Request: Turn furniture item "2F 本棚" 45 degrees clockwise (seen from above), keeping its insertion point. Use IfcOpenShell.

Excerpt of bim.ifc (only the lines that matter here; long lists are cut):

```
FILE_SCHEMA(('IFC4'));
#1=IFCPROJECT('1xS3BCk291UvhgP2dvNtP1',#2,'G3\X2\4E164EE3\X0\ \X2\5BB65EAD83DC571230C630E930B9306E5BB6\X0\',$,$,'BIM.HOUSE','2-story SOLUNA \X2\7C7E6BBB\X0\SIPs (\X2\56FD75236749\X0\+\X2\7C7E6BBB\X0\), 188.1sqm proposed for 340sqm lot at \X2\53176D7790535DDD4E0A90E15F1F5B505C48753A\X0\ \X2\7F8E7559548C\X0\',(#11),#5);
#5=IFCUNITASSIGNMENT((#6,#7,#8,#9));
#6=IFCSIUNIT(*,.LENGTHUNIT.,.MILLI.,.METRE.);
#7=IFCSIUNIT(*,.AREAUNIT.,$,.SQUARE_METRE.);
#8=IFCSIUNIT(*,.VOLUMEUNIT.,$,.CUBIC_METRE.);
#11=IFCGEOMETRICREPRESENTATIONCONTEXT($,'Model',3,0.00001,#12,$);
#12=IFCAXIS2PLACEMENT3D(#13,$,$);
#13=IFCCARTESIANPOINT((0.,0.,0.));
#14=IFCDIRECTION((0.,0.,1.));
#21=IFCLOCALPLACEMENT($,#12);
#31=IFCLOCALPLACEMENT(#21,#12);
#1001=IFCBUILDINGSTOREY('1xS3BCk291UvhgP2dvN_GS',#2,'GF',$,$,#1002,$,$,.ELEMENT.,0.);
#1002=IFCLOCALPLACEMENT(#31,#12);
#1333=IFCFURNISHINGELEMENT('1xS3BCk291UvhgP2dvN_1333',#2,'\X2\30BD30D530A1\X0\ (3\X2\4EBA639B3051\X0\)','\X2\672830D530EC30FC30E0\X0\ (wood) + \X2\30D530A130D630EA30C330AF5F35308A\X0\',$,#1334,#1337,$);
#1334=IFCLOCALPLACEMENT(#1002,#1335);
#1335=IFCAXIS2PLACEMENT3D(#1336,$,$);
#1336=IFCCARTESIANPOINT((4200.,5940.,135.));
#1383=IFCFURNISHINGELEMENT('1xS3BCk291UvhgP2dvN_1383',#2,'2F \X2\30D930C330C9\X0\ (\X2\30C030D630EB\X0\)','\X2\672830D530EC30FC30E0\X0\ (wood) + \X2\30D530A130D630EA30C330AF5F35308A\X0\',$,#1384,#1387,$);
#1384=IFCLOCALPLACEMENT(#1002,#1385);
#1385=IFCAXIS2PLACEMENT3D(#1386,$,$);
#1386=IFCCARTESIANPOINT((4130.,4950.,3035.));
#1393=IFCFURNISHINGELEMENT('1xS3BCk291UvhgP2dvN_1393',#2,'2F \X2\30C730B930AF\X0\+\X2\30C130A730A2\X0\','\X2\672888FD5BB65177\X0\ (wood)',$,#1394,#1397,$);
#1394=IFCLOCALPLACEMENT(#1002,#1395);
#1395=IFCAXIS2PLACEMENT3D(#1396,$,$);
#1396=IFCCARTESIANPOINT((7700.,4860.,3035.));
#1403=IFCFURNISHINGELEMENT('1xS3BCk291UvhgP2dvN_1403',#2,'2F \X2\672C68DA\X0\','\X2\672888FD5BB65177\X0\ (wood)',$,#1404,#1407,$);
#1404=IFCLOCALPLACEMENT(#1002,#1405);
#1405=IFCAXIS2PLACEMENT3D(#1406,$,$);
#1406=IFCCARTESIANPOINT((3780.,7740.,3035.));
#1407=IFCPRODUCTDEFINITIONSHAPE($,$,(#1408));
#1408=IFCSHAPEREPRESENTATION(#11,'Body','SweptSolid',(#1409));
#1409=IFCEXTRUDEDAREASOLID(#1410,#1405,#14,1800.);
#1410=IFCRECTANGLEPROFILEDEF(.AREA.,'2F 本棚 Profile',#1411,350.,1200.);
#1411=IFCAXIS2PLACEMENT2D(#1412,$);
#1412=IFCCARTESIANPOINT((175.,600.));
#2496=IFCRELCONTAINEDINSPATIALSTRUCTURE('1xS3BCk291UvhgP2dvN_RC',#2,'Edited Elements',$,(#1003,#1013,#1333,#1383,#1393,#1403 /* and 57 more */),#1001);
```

```python
import ifcopenshell
import ifcopenshell.api.geometry
import ifcopenshell.util.placement

model = ifcopenshell.open("bim.ifc")

item = model.by_id(1403)
matrix = ifcopenshell.util.placement.get_local_placement(item.ObjectPlacement)
matrix = matrix @ ifcopenshell.util.placement.rotation(-45, "Z")
ifcopenshell.api.geometry.edit_object_placement(model, product=item, matrix=matrix, is_si=False)

print(ifcopenshell.util.placement.get_local_placement(item.ObjectPlacement).round(3) + 0.0)

model.write("bim_rev.ifc")
```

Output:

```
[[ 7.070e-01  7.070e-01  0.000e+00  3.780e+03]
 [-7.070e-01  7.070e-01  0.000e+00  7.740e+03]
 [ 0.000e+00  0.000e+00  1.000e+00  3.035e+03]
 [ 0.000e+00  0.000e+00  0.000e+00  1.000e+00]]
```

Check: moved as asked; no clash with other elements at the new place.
